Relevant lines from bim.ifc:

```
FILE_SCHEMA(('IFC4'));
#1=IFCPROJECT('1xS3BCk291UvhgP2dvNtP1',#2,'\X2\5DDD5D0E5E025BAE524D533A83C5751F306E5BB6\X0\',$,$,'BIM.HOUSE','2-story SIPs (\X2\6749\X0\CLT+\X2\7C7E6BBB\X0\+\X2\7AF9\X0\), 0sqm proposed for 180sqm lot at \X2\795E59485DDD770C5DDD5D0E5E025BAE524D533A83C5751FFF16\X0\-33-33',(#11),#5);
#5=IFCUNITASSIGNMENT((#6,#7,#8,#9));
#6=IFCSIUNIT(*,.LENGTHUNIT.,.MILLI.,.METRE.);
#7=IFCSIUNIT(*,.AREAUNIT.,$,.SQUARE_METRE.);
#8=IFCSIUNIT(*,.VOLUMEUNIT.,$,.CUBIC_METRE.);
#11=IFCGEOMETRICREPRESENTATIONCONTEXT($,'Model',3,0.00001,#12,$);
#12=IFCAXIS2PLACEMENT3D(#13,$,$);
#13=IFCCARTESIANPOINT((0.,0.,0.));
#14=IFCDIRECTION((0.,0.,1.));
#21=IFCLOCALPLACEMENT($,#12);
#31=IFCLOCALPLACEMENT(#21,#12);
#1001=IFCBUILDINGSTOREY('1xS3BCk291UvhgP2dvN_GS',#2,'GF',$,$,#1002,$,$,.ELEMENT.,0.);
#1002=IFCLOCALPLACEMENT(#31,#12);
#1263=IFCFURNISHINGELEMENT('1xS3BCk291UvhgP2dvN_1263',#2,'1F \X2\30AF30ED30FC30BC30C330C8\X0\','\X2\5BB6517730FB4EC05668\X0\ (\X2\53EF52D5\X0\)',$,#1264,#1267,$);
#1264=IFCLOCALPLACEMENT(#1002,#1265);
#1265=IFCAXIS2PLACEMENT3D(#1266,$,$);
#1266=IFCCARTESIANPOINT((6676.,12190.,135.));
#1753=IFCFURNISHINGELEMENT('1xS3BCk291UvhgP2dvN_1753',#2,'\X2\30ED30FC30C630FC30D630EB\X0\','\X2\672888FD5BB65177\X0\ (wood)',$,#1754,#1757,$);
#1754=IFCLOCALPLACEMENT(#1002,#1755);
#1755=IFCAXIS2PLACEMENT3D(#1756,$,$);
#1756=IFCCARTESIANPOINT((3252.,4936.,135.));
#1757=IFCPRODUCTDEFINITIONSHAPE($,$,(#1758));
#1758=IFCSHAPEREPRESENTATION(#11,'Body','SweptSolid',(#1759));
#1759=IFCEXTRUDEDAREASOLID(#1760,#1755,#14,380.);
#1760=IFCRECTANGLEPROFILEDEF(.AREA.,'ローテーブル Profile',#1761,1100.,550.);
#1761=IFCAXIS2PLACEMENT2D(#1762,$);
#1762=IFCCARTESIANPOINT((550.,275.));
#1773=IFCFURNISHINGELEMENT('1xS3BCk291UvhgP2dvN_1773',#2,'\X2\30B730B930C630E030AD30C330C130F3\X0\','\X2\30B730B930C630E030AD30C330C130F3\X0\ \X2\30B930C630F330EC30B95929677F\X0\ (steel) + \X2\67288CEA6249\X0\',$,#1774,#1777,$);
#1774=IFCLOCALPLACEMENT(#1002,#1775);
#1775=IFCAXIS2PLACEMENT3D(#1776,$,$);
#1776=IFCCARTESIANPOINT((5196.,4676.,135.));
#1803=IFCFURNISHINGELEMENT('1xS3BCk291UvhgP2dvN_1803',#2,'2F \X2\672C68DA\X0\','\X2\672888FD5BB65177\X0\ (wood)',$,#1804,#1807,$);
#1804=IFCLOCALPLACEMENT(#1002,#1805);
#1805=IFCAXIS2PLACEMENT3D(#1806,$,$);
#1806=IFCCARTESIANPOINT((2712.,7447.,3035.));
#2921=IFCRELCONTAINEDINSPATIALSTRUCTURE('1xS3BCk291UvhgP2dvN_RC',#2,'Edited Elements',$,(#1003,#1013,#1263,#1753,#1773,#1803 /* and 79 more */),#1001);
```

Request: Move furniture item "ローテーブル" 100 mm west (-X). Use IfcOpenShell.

```python
import ifcopenshell
import ifcopenshell.api.geometry
import ifcopenshell.util.placement

model = ifcopenshell.open("bim.ifc")

item = model.by_guid("1xS3BCk291UvhgP2dvN_1753")
matrix = ifcopenshell.util.placement.get_local_placement(item.ObjectPlacement)
matrix[0, 3] -= 100.0
ifcopenshell.api.geometry.edit_object_placement(model, product=item, matrix=matrix, is_si=False)

print(ifcopenshell.util.placement.get_local_placement(item.ObjectPlacement).round(3) + 0.0)

model.write("bim-out.ifc")
```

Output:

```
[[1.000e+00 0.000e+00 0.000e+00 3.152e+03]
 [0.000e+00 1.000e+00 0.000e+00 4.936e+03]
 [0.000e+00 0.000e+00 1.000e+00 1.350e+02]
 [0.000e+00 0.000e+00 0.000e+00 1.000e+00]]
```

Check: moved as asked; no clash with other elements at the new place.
